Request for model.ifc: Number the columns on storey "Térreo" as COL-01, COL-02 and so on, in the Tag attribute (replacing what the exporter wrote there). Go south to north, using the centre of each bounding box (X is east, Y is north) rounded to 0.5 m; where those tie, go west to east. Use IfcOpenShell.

First a look at what the model holds.

```python
import ifcopenshell
import ifcopenshell.util.element
import ifcopenshell.util.placement

model = ifcopenshell.open("model.ifc")
print(model.schema)
storey = next(s for s in model.by_type("IfcBuildingStorey") if s.Name == "Térreo")
columns = [e for e in ifcopenshell.util.element.get_decomposition(storey) if e.is_a("IfcColumn")]
for e in sorted(columns, key=lambda e: e.id()):
    origin = ifcopenshell.util.placement.get_local_placement(e.ObjectPlacement)[:3, 3]
    print(e.id(), e.Tag, e.Name, origin.round(2) + 0.0, sep=" | ")
```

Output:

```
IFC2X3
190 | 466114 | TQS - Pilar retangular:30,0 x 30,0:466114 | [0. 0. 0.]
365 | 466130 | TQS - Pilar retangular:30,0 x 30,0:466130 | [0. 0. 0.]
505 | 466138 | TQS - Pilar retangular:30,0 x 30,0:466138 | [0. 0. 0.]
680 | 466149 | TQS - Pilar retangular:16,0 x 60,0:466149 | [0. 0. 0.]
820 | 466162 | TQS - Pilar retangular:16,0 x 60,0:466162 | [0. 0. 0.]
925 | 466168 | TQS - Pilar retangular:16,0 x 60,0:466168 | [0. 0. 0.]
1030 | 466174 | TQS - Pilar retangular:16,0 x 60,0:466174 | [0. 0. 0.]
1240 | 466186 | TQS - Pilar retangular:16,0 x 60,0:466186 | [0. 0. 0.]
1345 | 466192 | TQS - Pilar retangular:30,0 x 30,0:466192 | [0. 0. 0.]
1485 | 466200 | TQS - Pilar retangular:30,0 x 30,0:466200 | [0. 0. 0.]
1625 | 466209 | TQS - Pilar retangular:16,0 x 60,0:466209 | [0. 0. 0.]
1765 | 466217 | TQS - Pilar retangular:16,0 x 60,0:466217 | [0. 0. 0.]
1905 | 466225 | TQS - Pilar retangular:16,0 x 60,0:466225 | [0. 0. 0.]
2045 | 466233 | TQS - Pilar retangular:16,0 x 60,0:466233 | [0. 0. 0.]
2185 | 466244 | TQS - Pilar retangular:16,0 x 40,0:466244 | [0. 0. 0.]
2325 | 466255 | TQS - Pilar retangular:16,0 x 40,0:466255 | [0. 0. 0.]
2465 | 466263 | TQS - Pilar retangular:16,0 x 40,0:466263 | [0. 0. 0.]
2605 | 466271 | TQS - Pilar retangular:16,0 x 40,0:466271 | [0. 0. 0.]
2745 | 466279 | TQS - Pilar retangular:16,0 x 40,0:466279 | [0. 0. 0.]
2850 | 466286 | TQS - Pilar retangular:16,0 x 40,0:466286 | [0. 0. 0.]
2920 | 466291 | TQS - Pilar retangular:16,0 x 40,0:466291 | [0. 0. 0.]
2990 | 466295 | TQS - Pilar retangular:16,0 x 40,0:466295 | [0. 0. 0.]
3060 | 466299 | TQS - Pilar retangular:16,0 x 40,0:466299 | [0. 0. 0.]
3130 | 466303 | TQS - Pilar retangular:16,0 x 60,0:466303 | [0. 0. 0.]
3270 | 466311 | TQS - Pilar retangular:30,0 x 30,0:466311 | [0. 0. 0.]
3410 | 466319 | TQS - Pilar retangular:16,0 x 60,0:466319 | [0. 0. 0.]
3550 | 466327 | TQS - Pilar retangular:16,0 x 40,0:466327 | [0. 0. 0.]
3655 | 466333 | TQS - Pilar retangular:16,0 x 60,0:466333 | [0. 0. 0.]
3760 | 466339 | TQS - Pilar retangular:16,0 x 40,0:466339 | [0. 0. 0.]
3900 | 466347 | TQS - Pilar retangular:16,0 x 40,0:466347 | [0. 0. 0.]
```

```python
import ifcopenshell
import ifcopenshell.geom
import ifcopenshell.util.element
import ifcopenshell.util.shape

model = ifcopenshell.open("model.ifc")
settings = ifcopenshell.geom.settings()
settings.set("use-world-coords", True)


def centre(element):
    shape = ifcopenshell.geom.create_shape(settings, element)
    return ifcopenshell.util.shape.get_bbox_centroid(shape.geometry)


storey = next(s for s in model.by_type("IfcBuildingStorey") if s.Name == "Térreo")
columns = [e for e in ifcopenshell.util.element.get_decomposition(storey) if e.is_a("IfcColumn")]

# Insertion points can sit at a corner or the storey origin, so sort by the geometry (in metres).
centres = {e: centre(e) for e in columns}
columns.sort(key=lambda e: (round(centres[e][1] / 0.5), centres[e][0]))

for i, e in enumerate(columns, start=1):
    number = f"COL-{i:02d}"
    e.Tag = number
    print(e.id(), number)

model.write("model-out.ifc")
```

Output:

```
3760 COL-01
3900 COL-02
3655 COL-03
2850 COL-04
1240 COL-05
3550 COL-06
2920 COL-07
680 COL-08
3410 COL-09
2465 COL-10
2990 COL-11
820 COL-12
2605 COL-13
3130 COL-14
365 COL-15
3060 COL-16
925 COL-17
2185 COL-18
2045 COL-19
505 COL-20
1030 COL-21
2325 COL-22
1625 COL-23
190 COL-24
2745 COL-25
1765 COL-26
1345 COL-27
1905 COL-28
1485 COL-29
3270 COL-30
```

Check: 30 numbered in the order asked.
